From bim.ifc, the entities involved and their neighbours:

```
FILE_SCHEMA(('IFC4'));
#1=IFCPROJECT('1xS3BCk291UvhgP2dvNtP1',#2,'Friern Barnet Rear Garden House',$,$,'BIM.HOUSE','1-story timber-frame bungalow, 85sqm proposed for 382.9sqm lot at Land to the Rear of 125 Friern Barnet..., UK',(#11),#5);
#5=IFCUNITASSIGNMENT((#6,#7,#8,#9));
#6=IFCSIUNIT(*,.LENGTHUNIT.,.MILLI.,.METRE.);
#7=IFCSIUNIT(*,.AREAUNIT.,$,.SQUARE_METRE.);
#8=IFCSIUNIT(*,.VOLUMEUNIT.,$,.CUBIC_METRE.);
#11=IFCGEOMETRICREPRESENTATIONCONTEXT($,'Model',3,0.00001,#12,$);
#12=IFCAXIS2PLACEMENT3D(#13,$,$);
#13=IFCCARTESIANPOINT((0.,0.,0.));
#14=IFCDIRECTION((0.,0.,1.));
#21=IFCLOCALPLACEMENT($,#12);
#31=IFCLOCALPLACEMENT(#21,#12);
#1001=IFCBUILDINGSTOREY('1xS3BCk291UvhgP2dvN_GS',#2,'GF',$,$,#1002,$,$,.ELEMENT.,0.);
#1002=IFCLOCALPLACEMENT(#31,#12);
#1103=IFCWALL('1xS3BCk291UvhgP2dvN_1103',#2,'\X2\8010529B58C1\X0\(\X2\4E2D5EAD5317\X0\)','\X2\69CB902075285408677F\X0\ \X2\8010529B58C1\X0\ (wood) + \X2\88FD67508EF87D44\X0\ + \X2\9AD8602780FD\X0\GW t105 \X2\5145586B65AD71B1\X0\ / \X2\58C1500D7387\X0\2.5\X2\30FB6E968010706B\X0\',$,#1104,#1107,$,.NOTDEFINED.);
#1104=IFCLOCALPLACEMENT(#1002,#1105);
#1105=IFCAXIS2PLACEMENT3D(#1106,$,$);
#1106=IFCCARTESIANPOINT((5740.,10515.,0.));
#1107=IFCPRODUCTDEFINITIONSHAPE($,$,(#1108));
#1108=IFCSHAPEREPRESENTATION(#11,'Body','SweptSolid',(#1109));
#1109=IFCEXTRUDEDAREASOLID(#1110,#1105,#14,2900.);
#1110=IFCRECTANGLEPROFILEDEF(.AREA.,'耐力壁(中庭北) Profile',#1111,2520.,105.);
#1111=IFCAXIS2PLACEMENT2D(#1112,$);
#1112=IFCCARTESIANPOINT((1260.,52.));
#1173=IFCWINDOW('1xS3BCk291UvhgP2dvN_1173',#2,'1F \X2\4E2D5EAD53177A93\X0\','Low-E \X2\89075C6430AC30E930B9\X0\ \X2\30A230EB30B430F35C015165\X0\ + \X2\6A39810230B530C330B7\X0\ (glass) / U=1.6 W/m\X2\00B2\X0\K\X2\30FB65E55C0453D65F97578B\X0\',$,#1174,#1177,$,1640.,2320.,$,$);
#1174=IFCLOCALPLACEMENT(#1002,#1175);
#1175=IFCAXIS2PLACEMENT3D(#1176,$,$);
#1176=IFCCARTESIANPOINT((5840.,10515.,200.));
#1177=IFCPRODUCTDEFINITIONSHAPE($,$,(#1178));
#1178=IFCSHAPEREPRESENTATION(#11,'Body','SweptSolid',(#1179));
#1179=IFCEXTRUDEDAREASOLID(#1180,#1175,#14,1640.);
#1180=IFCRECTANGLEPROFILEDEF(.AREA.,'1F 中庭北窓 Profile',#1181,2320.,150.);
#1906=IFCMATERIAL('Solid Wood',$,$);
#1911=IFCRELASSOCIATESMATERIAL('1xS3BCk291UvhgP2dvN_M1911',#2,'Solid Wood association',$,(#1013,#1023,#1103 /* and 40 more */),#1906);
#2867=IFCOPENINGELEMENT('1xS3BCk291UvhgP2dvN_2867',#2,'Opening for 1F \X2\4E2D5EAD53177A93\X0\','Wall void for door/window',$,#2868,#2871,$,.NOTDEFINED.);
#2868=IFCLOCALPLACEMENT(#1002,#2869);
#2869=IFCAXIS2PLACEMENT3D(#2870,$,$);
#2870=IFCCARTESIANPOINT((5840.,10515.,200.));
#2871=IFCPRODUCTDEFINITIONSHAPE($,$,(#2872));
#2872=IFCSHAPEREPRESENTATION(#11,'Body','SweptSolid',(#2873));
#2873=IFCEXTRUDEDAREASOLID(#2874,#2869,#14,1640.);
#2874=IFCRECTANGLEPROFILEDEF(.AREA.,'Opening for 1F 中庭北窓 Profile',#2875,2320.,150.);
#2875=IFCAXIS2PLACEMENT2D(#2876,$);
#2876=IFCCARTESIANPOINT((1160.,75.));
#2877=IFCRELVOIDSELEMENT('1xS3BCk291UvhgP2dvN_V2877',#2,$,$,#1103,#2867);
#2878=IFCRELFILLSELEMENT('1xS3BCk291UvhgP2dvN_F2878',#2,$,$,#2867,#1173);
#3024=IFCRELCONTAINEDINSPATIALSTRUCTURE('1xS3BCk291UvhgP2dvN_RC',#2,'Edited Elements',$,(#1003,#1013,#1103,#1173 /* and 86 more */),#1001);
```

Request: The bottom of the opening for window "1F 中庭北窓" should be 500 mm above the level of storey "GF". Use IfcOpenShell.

```python
import numpy as np
import ifcopenshell
import ifcopenshell.api.geometry
import ifcopenshell.geom
import ifcopenshell.util.element
import ifcopenshell.util.placement
import ifcopenshell.util.shape
import ifcopenshell.util.unit

model = ifcopenshell.open("bim.ifc")
unit_scale = ifcopenshell.util.unit.calculate_unit_scale(model)

window = model.by_guid("1xS3BCk291UvhgP2dvN_1173")
opening = window.FillsVoids[0].RelatingOpeningElement
storey = ifcopenshell.util.element.get_container(window, ifc_class="IfcBuildingStorey")
level = ifcopenshell.util.placement.get_local_placement(storey.ObjectPlacement)[2, 3]

# The opening's origin need not be at the sill, so measure its lowest point.
shape = ifcopenshell.geom.create_shape(ifcopenshell.geom.settings(), opening)
bottom = ifcopenshell.util.shape.get_shape_bottom_elevation(shape, shape.geometry) / unit_scale
dz = level + 0.5 / unit_scale - bottom

shift = np.array([0.0, 0.0, dz])
# The window is not placed relative to its opening, so move both.
for product in (opening, window):
    matrix = ifcopenshell.util.placement.get_local_placement(product.ObjectPlacement)
    matrix[:3, 3] += shift
    ifcopenshell.api.geometry.edit_object_placement(model, product=product, matrix=matrix, is_si=False)

print(f"moved by {dz * unit_scale:+.3f} m")

model.write("bim_rev.ifc")
```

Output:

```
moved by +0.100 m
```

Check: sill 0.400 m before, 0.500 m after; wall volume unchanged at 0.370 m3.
